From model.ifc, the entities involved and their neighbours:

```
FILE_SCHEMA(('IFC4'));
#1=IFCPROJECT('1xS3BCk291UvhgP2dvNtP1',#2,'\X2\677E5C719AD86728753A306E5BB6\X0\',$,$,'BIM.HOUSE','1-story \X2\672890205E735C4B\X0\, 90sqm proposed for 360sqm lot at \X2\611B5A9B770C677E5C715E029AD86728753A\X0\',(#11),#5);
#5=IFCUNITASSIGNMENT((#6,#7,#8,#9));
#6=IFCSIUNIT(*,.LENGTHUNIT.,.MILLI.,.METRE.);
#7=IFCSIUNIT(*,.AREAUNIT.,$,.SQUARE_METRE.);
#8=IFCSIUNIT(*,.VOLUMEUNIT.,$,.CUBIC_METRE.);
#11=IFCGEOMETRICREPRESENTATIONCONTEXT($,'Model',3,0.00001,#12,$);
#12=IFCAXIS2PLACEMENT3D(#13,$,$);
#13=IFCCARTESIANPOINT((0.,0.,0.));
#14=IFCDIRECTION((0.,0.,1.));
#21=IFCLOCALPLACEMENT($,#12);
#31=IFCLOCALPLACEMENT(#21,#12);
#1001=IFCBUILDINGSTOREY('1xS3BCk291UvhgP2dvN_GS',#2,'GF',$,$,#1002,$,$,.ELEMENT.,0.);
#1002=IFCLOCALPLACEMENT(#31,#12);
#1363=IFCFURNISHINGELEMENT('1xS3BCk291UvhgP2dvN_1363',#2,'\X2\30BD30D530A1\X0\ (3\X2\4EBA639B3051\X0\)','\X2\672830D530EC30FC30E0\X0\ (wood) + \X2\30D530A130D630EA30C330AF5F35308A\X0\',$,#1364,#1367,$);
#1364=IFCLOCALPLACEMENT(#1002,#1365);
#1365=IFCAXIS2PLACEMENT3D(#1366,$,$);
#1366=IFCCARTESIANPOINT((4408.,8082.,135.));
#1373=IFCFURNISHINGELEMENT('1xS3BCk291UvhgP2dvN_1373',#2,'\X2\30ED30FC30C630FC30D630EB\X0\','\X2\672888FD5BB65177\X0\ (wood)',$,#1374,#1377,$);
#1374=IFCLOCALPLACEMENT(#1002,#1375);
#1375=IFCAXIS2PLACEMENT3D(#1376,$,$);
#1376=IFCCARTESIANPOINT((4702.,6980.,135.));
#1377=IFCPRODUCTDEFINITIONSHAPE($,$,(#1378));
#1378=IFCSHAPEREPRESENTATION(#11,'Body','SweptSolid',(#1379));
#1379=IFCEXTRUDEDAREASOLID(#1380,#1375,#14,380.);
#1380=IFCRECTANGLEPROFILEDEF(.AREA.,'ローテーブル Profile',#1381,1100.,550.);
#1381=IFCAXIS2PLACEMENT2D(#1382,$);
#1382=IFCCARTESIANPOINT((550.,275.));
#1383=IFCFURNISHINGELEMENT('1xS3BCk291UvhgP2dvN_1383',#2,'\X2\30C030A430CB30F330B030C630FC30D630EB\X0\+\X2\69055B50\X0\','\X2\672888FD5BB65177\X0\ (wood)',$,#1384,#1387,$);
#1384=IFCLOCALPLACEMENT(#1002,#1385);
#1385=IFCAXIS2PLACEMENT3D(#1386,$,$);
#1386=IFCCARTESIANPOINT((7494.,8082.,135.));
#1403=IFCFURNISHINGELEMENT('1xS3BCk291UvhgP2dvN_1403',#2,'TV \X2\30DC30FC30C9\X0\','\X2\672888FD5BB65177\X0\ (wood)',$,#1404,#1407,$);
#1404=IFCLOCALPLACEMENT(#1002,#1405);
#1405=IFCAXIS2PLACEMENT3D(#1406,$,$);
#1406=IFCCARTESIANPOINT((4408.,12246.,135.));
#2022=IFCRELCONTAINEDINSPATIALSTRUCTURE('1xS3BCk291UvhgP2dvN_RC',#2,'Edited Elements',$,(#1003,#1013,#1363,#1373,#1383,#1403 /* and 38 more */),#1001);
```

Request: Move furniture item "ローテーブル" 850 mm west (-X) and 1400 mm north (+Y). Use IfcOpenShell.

```python
import ifcopenshell
import ifcopenshell.api.geometry
import ifcopenshell.util.placement
import ifcopenshell.util.unit

model = ifcopenshell.open("model.ifc")
unit_scale = ifcopenshell.util.unit.calculate_unit_scale(model)

item = model.by_guid("1xS3BCk291UvhgP2dvN_1373")
matrix = ifcopenshell.util.placement.get_local_placement(item.ObjectPlacement)
matrix[0, 3] -= 0.85 / unit_scale
matrix[1, 3] += 1.4 / unit_scale
ifcopenshell.api.geometry.edit_object_placement(model, product=item, matrix=matrix, is_si=False)

print(ifcopenshell.util.placement.get_local_placement(item.ObjectPlacement).round(3) + 0.0)

model.write("model_v2.ifc")
```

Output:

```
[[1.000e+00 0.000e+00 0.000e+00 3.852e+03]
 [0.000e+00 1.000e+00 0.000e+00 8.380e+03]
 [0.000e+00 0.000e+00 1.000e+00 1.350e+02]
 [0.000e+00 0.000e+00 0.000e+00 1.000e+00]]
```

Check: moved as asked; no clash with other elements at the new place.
